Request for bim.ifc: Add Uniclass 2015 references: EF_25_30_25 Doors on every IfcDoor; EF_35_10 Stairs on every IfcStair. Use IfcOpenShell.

First a look at what the model holds.

```python
import ifcopenshell

model = ifcopenshell.open("bim.ifc")
print(model.schema)
print("classifications:", [c.Name for c in model.by_type("IfcClassification")])
for ifc_class in ("IfcDoor", "IfcRoof", "IfcStair", "IfcWall", "IfcWindow"):
    print(ifc_class, len(model.by_type(ifc_class)))
```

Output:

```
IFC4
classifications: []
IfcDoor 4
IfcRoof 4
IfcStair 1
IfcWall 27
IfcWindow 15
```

```python
import ifcopenshell
import ifcopenshell.api.classification

model = ifcopenshell.open("bim.ifc")

system = ifcopenshell.api.classification.add_classification(model, classification="Uniclass 2015")

codes = {
    "IfcDoor": ("EF_25_30_25", "Doors"),
    "IfcStair": ("EF_35_10", "Stairs"),
}
for ifc_class, (code, name) in codes.items():
    products = model.by_type(ifc_class)
    ifcopenshell.api.classification.add_reference(
        model, products=products, classification=system, identification=code, name=name
    )
    print(code, len(products))

model.write("bim_v2.ifc")
```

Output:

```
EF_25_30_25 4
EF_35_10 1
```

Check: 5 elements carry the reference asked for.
